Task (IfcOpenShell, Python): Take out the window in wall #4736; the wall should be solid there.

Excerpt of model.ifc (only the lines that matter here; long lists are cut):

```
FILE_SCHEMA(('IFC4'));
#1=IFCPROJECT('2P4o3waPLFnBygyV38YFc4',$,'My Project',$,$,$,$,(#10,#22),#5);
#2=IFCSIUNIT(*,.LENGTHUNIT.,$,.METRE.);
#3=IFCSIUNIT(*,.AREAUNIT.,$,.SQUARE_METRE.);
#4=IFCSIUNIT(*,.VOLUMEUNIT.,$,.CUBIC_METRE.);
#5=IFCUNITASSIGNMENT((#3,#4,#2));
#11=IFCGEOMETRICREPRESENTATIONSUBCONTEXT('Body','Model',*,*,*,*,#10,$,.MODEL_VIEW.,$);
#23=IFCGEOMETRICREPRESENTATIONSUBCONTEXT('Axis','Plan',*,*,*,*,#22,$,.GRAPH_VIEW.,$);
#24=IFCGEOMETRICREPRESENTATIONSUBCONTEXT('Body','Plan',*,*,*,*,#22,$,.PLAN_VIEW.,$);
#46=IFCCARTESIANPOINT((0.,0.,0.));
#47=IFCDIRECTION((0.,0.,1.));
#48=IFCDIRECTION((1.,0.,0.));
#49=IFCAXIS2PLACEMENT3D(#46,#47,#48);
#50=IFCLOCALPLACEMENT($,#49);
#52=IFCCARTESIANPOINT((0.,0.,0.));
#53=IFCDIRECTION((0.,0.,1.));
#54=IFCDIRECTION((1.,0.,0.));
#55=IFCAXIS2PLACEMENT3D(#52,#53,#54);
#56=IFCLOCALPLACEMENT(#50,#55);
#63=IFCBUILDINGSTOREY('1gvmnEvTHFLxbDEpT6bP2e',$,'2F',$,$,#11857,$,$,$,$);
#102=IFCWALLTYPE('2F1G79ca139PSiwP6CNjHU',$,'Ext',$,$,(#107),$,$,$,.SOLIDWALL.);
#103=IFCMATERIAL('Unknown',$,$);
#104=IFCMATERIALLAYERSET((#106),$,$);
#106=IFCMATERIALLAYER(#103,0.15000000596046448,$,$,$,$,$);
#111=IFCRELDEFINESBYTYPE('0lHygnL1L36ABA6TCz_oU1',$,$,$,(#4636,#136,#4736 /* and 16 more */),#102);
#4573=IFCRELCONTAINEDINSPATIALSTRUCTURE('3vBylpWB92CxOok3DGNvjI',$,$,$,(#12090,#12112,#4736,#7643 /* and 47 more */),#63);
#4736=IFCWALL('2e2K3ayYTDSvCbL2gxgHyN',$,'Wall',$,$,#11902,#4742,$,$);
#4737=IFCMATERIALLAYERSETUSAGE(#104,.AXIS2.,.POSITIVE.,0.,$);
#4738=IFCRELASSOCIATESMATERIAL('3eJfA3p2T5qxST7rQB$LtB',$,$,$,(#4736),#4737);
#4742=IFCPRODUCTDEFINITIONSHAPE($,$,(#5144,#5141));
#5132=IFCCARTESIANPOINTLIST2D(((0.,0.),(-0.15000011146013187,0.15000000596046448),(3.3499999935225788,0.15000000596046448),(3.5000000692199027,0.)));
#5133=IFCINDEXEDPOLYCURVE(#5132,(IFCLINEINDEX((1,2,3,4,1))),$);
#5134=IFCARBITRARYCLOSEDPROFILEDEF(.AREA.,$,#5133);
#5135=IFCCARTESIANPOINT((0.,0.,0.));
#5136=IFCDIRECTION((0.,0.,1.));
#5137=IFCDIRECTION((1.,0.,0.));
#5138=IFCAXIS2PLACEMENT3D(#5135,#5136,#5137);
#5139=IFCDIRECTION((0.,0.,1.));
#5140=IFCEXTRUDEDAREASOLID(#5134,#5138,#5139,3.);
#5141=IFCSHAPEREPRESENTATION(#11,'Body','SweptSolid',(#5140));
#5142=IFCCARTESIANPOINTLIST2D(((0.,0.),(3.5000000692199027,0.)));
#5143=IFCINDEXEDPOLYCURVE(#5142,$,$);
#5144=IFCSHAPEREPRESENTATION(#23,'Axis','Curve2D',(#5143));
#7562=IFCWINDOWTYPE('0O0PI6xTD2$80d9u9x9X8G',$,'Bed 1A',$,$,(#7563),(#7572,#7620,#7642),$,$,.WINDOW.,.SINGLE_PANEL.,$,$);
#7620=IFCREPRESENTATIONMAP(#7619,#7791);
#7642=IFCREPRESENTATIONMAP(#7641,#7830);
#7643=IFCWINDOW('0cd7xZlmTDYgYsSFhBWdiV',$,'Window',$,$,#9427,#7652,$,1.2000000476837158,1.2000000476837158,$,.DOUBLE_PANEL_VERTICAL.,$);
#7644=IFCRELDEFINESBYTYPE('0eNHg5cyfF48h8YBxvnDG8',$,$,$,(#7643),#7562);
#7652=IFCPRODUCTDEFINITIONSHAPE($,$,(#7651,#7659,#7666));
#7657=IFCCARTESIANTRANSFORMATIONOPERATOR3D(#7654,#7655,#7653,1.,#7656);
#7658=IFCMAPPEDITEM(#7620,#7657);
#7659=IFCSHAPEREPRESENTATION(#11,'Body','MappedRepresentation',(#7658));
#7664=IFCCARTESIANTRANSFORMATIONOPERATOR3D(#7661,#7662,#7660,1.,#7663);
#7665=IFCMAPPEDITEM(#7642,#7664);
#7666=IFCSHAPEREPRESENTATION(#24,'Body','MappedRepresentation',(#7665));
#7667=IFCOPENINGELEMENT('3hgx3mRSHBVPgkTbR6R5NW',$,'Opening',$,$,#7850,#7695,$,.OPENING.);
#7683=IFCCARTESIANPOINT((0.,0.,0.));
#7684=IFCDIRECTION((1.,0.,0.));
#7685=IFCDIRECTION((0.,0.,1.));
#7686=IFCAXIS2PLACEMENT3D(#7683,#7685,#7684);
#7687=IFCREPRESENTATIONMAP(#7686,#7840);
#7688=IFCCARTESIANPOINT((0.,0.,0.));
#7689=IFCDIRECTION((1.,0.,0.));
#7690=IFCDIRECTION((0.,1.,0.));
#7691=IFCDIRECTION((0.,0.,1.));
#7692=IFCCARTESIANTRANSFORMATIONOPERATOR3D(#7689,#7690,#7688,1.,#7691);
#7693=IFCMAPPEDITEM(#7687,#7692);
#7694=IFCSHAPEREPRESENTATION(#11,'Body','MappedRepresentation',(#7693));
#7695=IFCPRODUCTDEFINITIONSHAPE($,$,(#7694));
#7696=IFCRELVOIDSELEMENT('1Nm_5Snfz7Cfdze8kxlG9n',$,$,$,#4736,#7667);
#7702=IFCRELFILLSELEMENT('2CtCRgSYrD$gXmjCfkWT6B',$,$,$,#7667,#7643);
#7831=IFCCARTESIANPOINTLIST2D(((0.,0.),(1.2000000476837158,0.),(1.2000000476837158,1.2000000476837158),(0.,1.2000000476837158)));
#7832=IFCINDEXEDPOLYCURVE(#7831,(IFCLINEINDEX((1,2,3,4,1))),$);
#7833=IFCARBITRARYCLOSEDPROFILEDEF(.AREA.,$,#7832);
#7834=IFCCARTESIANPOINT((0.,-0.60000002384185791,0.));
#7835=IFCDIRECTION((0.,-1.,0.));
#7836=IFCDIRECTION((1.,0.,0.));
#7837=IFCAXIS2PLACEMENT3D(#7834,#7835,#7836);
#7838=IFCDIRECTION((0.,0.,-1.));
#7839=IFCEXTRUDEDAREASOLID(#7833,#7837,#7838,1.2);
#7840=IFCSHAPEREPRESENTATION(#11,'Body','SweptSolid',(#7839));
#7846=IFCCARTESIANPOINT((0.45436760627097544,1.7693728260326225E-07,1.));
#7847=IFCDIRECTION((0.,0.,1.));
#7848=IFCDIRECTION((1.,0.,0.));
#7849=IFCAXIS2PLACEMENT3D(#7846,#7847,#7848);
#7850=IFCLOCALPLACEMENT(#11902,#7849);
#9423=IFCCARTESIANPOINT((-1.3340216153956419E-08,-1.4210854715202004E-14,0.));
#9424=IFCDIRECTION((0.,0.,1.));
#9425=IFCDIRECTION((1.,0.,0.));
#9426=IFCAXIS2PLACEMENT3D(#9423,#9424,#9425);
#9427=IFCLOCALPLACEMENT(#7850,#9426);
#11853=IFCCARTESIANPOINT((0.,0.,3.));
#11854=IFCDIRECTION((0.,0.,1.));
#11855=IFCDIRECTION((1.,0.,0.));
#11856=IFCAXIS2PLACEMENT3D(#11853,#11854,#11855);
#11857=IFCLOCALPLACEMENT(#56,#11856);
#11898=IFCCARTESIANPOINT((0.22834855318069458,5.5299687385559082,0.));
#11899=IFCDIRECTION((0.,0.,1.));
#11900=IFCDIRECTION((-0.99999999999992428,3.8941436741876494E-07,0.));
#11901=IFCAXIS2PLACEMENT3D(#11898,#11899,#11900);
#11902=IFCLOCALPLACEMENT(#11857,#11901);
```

```python
import ifcopenshell
import ifcopenshell.api.feature
import ifcopenshell.api.root
import ifcopenshell.geom
import ifcopenshell.util.shape

model = ifcopenshell.open("model.ifc")
settings = ifcopenshell.geom.settings()


def volume(element):
    """Net volume in cubic metres, openings subtracted."""
    shape = ifcopenshell.geom.create_shape(settings, element)
    return ifcopenshell.util.shape.get_volume(shape.geometry)


window = model.by_id(7643)
opening = window.FillsVoids[0].RelatingOpeningElement
wall = opening.VoidsElements[0].RelatingBuildingElement
before = volume(wall)

ifcopenshell.api.root.remove_product(model, product=window)
ifcopenshell.api.feature.remove_feature(model, feature=opening)

after = volume(wall)

print(f"wall volume {before:.3f} -> {after:.3f} m3")

model.write("model_updated.ifc")
```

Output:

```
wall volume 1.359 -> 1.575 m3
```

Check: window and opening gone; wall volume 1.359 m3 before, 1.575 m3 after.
